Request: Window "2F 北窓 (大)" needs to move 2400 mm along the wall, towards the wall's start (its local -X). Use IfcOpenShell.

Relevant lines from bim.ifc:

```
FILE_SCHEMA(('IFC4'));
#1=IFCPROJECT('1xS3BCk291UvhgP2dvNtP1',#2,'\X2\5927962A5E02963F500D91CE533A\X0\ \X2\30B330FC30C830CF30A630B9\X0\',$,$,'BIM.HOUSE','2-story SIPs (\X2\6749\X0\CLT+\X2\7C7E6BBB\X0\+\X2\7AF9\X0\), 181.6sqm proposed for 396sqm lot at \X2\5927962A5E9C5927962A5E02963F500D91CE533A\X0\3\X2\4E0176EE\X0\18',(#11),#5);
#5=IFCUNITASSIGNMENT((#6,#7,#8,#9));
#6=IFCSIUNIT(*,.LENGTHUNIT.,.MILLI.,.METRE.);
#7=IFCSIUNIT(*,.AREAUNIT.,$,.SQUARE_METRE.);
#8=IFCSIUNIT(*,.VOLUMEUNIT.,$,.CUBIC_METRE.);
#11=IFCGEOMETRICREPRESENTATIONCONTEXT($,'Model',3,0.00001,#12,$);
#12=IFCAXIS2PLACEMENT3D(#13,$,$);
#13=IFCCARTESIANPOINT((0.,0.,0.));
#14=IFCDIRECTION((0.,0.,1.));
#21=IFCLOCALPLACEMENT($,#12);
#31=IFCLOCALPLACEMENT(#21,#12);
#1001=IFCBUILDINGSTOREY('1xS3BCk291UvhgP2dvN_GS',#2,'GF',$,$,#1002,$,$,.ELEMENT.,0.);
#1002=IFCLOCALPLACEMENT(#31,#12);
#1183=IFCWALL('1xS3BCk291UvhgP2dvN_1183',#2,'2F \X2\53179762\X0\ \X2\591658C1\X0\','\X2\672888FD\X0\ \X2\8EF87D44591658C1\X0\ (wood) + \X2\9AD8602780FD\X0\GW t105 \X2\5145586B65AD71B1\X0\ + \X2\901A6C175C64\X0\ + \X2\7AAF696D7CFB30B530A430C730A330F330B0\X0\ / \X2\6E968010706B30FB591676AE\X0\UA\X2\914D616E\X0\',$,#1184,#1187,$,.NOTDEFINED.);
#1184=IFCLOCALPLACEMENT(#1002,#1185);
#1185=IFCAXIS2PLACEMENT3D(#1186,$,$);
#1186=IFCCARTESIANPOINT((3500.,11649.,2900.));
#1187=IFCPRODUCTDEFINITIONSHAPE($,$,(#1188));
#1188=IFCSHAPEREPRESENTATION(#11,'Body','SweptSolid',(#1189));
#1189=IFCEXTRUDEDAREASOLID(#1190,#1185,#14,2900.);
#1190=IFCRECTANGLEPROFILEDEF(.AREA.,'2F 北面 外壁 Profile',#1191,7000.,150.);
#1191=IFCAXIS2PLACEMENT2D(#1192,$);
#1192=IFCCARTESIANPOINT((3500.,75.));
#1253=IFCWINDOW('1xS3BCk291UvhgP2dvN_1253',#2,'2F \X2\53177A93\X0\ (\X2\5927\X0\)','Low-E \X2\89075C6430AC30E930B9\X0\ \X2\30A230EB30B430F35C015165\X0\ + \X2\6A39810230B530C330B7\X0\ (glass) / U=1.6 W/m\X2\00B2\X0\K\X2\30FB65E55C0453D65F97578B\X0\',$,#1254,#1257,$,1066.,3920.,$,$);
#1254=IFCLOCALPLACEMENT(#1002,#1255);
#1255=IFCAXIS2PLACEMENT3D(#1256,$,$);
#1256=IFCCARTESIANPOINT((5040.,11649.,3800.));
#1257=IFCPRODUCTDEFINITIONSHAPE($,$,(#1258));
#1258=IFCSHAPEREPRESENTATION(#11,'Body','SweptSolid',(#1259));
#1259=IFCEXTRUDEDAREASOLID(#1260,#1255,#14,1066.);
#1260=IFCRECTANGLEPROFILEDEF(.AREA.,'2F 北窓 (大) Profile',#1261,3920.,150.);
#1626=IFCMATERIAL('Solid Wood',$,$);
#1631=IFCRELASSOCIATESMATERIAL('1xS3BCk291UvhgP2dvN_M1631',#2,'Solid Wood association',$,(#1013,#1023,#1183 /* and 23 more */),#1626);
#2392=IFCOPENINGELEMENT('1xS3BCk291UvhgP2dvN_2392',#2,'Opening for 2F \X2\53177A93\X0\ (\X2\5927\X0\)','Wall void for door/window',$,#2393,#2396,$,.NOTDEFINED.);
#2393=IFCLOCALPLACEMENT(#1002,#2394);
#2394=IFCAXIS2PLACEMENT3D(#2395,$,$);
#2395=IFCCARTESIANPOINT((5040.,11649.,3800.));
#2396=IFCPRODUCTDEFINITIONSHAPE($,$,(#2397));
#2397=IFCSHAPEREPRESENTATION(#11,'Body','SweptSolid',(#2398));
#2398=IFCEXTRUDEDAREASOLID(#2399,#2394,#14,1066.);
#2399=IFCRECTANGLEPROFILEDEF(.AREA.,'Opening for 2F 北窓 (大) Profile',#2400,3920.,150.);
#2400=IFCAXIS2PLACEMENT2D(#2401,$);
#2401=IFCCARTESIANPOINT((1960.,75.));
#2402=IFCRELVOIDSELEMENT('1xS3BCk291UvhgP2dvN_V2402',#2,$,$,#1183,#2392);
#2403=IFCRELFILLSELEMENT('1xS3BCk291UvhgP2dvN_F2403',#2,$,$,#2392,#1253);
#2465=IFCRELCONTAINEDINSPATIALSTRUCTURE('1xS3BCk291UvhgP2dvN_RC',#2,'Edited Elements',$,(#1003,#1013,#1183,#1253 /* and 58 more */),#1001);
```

```python
import ifcopenshell
import ifcopenshell.api.geometry
import ifcopenshell.util.placement
import ifcopenshell.util.unit

model = ifcopenshell.open("bim.ifc")
unit_scale = ifcopenshell.util.unit.calculate_unit_scale(model)

window = model.by_guid("1xS3BCk291UvhgP2dvN_1253")
opening = window.FillsVoids[0].RelatingOpeningElement
wall = opening.VoidsElements[0].RelatingBuildingElement

wall_matrix = ifcopenshell.util.placement.get_local_placement(wall.ObjectPlacement)
shift = wall_matrix[:3, 0] * -2.4 / unit_scale
before = ifcopenshell.util.placement.get_local_placement(window.ObjectPlacement)[:3, 3].copy()

# The window is not placed relative to its opening, so move both.
for product in (opening, window):
    matrix = ifcopenshell.util.placement.get_local_placement(product.ObjectPlacement)
    matrix[:3, 3] += shift
    ifcopenshell.api.geometry.edit_object_placement(model, product=product, matrix=matrix, is_si=False)

after = ifcopenshell.util.placement.get_local_placement(window.ObjectPlacement)[:3, 3]
print("window moved by", (after - before).round(3) + 0.0)

model.write("bim_v2.ifc")
```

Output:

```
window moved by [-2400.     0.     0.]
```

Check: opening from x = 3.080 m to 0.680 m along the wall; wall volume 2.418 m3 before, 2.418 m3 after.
